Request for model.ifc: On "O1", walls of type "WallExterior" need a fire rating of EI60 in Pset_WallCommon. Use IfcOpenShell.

First a look at what the model holds.

```python
import ifcopenshell
import ifcopenshell.util.element

model = ifcopenshell.open("model.ifc")
print(model.schema)
storey = next(s for s in model.by_type("IfcBuildingStorey") if s.Name == "O1")
walls = [e for e in ifcopenshell.util.element.get_decomposition(storey) if e.is_a("IfcWall")]
seen = {}
for e in walls:
    element_type = ifcopenshell.util.element.get_type(e)
    key = (element_type.Name if element_type != e and element_type else None, ifcopenshell.util.element.get_pset(e, "Pset_WallCommon", "FireRating"))
    seen[key] = seen.get(key, 0) + 1
for (name, value), count in sorted(seen.items(), key=str):
    print(count, "x", name, "|", value)
```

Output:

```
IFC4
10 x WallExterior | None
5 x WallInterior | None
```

```python
import ifcopenshell
import ifcopenshell.api.pset
import ifcopenshell.util.element

model = ifcopenshell.open("model.ifc")

storey = next(s for s in model.by_type("IfcBuildingStorey") if s.Name == "O1")
walls = [e for e in ifcopenshell.util.element.get_decomposition(storey) if e.is_a("IfcWall")]

count = 0
for e in walls:
    element_type = ifcopenshell.util.element.get_type(e)
    if element_type in (None, e) or element_type.Name != "WallExterior":
        continue
    # add_pset returns the element's existing set when there is one.
    pset = ifcopenshell.api.pset.add_pset(model, product=e, name="Pset_WallCommon")
    ifcopenshell.api.pset.edit_pset(model, pset=pset, properties={"FireRating": "EI60"})
    count += 1

print(count, "walls updated")

model.write("model_updated.ifc")
```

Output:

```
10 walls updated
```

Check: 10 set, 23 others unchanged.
